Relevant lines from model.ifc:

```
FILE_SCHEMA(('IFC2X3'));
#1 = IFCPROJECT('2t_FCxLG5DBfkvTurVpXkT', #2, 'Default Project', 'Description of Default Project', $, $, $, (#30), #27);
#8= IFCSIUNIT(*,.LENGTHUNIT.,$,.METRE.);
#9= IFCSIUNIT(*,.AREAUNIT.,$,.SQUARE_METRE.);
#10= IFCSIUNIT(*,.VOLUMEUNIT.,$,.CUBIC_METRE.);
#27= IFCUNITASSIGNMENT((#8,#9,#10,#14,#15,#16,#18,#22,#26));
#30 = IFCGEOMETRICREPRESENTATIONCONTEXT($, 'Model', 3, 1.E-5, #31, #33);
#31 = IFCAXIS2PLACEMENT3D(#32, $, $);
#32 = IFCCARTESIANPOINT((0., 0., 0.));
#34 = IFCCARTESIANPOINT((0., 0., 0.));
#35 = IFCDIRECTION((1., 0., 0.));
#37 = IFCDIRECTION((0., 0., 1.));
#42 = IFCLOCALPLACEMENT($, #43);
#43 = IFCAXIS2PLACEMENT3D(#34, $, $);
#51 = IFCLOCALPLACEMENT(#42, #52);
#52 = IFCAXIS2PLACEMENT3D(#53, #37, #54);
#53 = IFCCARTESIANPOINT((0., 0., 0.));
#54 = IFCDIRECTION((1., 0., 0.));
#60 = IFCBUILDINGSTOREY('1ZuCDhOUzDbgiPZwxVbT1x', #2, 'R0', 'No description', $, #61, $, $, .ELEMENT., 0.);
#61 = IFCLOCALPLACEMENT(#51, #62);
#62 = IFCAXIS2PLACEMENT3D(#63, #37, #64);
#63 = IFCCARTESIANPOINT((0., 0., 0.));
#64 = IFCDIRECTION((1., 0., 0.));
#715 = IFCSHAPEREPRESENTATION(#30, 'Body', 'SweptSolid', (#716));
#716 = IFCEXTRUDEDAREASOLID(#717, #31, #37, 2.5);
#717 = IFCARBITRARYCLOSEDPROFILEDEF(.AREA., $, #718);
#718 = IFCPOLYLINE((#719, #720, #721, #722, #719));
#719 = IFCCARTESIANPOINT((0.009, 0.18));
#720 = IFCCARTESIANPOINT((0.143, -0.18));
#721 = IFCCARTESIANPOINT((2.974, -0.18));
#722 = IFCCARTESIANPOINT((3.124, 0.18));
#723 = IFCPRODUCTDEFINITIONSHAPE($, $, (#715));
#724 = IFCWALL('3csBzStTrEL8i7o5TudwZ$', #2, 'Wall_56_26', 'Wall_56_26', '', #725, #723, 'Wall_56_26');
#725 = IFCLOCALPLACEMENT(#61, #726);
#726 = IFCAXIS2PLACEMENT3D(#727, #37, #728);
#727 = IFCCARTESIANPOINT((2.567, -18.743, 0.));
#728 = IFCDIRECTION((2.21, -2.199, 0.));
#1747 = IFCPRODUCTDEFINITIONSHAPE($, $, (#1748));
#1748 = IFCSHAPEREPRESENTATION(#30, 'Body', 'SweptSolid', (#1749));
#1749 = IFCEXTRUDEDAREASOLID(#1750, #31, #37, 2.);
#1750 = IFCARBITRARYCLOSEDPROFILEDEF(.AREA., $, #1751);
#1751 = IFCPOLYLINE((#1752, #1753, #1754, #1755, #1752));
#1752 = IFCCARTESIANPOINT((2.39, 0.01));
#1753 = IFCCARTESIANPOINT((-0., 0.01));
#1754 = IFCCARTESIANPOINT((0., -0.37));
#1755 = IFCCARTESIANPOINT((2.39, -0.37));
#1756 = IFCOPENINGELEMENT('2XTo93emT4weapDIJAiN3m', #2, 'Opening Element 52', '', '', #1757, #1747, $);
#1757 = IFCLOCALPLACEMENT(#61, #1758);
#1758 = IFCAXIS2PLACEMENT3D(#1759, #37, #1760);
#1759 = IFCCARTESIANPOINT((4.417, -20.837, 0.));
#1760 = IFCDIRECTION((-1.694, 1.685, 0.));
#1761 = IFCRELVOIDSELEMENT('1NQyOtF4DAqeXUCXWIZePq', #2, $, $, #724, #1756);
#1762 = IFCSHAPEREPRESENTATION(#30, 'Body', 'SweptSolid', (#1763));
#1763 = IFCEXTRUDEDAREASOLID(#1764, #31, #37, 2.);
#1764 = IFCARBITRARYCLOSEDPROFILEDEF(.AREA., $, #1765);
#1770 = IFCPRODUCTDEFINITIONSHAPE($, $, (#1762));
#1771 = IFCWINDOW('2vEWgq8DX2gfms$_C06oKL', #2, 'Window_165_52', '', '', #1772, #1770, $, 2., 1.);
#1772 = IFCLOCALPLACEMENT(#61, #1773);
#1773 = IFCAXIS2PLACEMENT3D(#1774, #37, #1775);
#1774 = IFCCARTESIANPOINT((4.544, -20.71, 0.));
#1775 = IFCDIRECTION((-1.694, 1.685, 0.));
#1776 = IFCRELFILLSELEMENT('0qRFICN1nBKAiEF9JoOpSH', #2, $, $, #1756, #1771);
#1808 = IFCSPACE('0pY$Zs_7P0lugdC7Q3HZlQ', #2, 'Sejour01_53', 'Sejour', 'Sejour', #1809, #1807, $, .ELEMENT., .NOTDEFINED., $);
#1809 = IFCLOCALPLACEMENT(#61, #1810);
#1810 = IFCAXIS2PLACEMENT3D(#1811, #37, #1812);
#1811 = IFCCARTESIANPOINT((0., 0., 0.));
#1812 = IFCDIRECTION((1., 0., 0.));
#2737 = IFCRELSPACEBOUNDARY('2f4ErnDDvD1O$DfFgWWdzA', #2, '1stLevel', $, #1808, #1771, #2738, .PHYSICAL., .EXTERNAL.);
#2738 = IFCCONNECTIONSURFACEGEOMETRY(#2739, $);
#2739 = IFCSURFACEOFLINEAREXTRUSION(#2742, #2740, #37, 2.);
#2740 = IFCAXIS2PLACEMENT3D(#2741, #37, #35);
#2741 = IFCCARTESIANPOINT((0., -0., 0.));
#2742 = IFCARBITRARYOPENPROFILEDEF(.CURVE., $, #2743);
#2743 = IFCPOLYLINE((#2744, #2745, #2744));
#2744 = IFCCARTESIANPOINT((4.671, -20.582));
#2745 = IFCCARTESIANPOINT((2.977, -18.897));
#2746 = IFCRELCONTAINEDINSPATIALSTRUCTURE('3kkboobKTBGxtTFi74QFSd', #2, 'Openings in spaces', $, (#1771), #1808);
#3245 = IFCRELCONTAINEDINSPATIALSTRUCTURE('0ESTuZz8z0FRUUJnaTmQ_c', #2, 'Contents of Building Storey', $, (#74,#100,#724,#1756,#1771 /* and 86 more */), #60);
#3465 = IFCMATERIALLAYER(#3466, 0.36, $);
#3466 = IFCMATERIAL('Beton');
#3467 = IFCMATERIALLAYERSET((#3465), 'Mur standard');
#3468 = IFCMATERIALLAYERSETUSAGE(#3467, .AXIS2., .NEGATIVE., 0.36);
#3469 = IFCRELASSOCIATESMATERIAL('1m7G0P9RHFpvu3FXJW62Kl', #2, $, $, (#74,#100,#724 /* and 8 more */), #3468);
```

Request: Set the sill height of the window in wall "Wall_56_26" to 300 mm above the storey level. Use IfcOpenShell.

```python
import numpy as np
import ifcopenshell
import ifcopenshell.api.geometry
import ifcopenshell.geom
import ifcopenshell.util.element
import ifcopenshell.util.placement
import ifcopenshell.util.shape
import ifcopenshell.util.unit

model = ifcopenshell.open("model.ifc")
unit_scale = ifcopenshell.util.unit.calculate_unit_scale(model)

window = model.by_guid("2vEWgq8DX2gfms$_C06oKL")
opening = window.FillsVoids[0].RelatingOpeningElement
storey = ifcopenshell.util.element.get_container(window, ifc_class="IfcBuildingStorey")
level = ifcopenshell.util.placement.get_local_placement(storey.ObjectPlacement)[2, 3]

# The opening's origin need not be at the sill, so measure its lowest point.
shape = ifcopenshell.geom.create_shape(ifcopenshell.geom.settings(), opening)
bottom = ifcopenshell.util.shape.get_shape_bottom_elevation(shape, shape.geometry) / unit_scale
dz = level + 0.3 / unit_scale - bottom

shift = np.array([0.0, 0.0, dz])
# The window is not placed relative to its opening, so move both.
for product in (opening, window):
    matrix = ifcopenshell.util.placement.get_local_placement(product.ObjectPlacement)
    matrix[:3, 3] += shift
    ifcopenshell.api.geometry.edit_object_placement(model, product=product, matrix=matrix, is_si=False)

# Space boundary surfaces are stored in each space's coordinates; move them too.
for rel in window.ProvidesBoundaries:
    if not rel.ConnectionGeometry:
        continue
    surface = rel.ConnectionGeometry.SurfaceOnRelatingElement
    space_matrix = ifcopenshell.util.placement.get_local_placement(rel.RelatingSpace.ObjectPlacement)
    point = np.array(surface.Position.Location.Coordinates) + space_matrix[:3, :3].T @ shift
    surface.Position = model.createIfcAxis2Placement3D(
        model.createIfcCartesianPoint(point.tolist()), surface.Position.Axis, surface.Position.RefDirection
    )

print(f"moved by {dz * unit_scale:+.3f} m")

model.write("model_v2.ifc")
```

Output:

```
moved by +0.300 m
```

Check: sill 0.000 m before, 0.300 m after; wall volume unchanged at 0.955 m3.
